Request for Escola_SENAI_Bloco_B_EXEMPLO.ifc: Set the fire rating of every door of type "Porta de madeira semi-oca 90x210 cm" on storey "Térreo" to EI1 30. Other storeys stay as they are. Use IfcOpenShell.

First a look at what the model holds.

```python
import ifcopenshell
import ifcopenshell.util.element

model = ifcopenshell.open("Escola_SENAI_Bloco_B_EXEMPLO.ifc")
print(model.schema)
storey = next(s for s in model.by_type("IfcBuildingStorey") if s.Name == "Térreo")
doors = [e for e in ifcopenshell.util.element.get_decomposition(storey) if e.is_a("IfcDoor")]
seen = {}
for e in doors:
    element_type = ifcopenshell.util.element.get_type(e)
    key = (element_type.Name if element_type != e and element_type else None, ifcopenshell.util.element.get_pset(e, "Pset_DoorCommon", "FireRating"))
    seen[key] = seen.get(key, 0) + 1
for (name, value), count in sorted(seen.items(), key=str):
    print(count, "x", name, "|", value)
```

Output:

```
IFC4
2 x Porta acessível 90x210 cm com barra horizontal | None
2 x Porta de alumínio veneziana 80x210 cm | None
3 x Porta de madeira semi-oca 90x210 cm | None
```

```python
import ifcopenshell
import ifcopenshell.api.pset
import ifcopenshell.util.element

model = ifcopenshell.open("Escola_SENAI_Bloco_B_EXEMPLO.ifc")

storey = next(s for s in model.by_type("IfcBuildingStorey") if s.Name == "Térreo")
doors = [e for e in ifcopenshell.util.element.get_decomposition(storey) if e.is_a("IfcDoor")]

count = 0
for e in doors:
    element_type = ifcopenshell.util.element.get_type(e)
    if element_type in (None, e) or element_type.Name != "Porta de madeira semi-oca 90x210 cm":
        continue
    # add_pset returns the element's existing set when there is one.
    pset = ifcopenshell.api.pset.add_pset(model, product=e, name="Pset_DoorCommon")
    ifcopenshell.api.pset.edit_pset(model, pset=pset, properties={"FireRating": "EI1 30"})
    count += 1

print(count, "doors updated")

model.write("Escola_SENAI_Bloco_B_EXEMPLO_updated.ifc")
```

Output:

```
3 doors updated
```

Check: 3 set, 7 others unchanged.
